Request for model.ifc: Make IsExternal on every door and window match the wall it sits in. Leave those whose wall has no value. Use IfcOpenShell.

First a look at what the model holds.

```python
import ifcopenshell
import ifcopenshell.util.element

model = ifcopenshell.open("model.ifc")
print(model.schema)
seen = {}
for e in model.by_type("IfcDoor") + model.by_type("IfcWindow"):
    if not e.FillsVoids:
        continue
    host = e.FillsVoids[0].RelatingOpeningElement.VoidsElements[0].RelatingBuildingElement
    own = ifcopenshell.util.element.get_pset(e, f"Pset_{e.is_a()[3:].removesuffix('StandardCase')}Common", "IsExternal")
    wall = ifcopenshell.util.element.get_pset(host, "Pset_WallCommon", "IsExternal")
    seen[e.is_a(), own, wall] = seen.get((e.is_a(), own, wall), 0) + 1
for (cls, own, wall), count in sorted(seen.items(), key=str):
    print(count, cls, "IsExternal:", own, "| host wall:", wall)
```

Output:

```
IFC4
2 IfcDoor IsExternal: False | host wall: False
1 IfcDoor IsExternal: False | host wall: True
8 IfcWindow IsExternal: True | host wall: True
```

```python
import ifcopenshell
import ifcopenshell.api.pset
import ifcopenshell.util.element

model = ifcopenshell.open("model.ifc")

count = 0
for ifc_class, pset_name in (("IfcDoor", "Pset_DoorCommon"), ("IfcWindow", "Pset_WindowCommon")):
    for e in model.by_type(ifc_class):
        if not e.FillsVoids:
            continue
        host = e.FillsVoids[0].RelatingOpeningElement.VoidsElements[0].RelatingBuildingElement
        external = ifcopenshell.util.element.get_pset(host, "Pset_WallCommon", "IsExternal")
        if external is None or ifcopenshell.util.element.get_pset(e, pset_name, "IsExternal") == external:
            continue
        pset = ifcopenshell.api.pset.add_pset(model, product=e, name=pset_name)
        ifcopenshell.api.pset.edit_pset(model, pset=pset, properties={"IsExternal": external})
        count += 1

print(count, "updated")

model.write("model-out.ifc")
```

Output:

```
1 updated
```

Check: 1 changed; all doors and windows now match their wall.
